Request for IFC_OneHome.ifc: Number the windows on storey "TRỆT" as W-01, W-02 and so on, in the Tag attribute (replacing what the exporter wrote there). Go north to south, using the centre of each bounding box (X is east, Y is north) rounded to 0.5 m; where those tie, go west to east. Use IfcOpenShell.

First a look at what the model holds.

```python
import ifcopenshell
import ifcopenshell.util.element
import ifcopenshell.util.placement

model = ifcopenshell.open("IFC_OneHome.ifc")
print(model.schema)
storey = next(s for s in model.by_type("IfcBuildingStorey") if s.Name == "TRỆT")
windows = [e for e in ifcopenshell.util.element.get_decomposition(storey) if e.is_a("IfcWindow")]
for e in sorted(windows, key=lambda e: e.id()):
    origin = ifcopenshell.util.placement.get_local_placement(e.ObjectPlacement)[:3, 3]
    print(e.id(), e.Tag, e.Name, origin.round(2) + 0.0, sep=" | ")
```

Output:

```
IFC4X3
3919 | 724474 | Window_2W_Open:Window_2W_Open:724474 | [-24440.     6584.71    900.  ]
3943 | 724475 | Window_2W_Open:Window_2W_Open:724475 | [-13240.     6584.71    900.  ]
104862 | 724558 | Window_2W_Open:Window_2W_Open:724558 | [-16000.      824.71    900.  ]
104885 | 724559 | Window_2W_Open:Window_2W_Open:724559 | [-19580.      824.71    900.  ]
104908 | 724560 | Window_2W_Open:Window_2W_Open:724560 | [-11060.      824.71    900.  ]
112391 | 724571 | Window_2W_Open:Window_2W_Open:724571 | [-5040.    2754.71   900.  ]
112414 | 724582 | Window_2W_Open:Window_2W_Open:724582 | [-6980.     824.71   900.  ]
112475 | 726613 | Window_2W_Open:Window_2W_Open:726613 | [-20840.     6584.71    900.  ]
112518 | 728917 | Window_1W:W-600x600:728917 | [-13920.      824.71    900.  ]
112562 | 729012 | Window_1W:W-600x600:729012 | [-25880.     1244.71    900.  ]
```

```python
import ifcopenshell
import ifcopenshell.geom
import ifcopenshell.util.element
import ifcopenshell.util.shape

model = ifcopenshell.open("IFC_OneHome.ifc")
settings = ifcopenshell.geom.settings()
settings.set("use-world-coords", True)


def centre(element):
    shape = ifcopenshell.geom.create_shape(settings, element)
    return ifcopenshell.util.shape.get_bbox_centroid(shape.geometry)


storey = next(s for s in model.by_type("IfcBuildingStorey") if s.Name == "TRỆT")
windows = [e for e in ifcopenshell.util.element.get_decomposition(storey) if e.is_a("IfcWindow")]

# Insertion points can sit at a corner or the storey origin, so sort by the geometry (in metres).
centres = {e: centre(e) for e in windows}
windows.sort(key=lambda e: (-round(centres[e][1] / 0.5), centres[e][0]))

for i, e in enumerate(windows, start=1):
    number = f"W-{i:02d}"
    e.Tag = number
    print(e.id(), number)

model.write("IFC_OneHome_edited.ifc")
```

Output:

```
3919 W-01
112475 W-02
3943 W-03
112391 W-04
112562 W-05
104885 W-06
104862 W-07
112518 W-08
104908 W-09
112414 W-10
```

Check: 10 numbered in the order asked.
